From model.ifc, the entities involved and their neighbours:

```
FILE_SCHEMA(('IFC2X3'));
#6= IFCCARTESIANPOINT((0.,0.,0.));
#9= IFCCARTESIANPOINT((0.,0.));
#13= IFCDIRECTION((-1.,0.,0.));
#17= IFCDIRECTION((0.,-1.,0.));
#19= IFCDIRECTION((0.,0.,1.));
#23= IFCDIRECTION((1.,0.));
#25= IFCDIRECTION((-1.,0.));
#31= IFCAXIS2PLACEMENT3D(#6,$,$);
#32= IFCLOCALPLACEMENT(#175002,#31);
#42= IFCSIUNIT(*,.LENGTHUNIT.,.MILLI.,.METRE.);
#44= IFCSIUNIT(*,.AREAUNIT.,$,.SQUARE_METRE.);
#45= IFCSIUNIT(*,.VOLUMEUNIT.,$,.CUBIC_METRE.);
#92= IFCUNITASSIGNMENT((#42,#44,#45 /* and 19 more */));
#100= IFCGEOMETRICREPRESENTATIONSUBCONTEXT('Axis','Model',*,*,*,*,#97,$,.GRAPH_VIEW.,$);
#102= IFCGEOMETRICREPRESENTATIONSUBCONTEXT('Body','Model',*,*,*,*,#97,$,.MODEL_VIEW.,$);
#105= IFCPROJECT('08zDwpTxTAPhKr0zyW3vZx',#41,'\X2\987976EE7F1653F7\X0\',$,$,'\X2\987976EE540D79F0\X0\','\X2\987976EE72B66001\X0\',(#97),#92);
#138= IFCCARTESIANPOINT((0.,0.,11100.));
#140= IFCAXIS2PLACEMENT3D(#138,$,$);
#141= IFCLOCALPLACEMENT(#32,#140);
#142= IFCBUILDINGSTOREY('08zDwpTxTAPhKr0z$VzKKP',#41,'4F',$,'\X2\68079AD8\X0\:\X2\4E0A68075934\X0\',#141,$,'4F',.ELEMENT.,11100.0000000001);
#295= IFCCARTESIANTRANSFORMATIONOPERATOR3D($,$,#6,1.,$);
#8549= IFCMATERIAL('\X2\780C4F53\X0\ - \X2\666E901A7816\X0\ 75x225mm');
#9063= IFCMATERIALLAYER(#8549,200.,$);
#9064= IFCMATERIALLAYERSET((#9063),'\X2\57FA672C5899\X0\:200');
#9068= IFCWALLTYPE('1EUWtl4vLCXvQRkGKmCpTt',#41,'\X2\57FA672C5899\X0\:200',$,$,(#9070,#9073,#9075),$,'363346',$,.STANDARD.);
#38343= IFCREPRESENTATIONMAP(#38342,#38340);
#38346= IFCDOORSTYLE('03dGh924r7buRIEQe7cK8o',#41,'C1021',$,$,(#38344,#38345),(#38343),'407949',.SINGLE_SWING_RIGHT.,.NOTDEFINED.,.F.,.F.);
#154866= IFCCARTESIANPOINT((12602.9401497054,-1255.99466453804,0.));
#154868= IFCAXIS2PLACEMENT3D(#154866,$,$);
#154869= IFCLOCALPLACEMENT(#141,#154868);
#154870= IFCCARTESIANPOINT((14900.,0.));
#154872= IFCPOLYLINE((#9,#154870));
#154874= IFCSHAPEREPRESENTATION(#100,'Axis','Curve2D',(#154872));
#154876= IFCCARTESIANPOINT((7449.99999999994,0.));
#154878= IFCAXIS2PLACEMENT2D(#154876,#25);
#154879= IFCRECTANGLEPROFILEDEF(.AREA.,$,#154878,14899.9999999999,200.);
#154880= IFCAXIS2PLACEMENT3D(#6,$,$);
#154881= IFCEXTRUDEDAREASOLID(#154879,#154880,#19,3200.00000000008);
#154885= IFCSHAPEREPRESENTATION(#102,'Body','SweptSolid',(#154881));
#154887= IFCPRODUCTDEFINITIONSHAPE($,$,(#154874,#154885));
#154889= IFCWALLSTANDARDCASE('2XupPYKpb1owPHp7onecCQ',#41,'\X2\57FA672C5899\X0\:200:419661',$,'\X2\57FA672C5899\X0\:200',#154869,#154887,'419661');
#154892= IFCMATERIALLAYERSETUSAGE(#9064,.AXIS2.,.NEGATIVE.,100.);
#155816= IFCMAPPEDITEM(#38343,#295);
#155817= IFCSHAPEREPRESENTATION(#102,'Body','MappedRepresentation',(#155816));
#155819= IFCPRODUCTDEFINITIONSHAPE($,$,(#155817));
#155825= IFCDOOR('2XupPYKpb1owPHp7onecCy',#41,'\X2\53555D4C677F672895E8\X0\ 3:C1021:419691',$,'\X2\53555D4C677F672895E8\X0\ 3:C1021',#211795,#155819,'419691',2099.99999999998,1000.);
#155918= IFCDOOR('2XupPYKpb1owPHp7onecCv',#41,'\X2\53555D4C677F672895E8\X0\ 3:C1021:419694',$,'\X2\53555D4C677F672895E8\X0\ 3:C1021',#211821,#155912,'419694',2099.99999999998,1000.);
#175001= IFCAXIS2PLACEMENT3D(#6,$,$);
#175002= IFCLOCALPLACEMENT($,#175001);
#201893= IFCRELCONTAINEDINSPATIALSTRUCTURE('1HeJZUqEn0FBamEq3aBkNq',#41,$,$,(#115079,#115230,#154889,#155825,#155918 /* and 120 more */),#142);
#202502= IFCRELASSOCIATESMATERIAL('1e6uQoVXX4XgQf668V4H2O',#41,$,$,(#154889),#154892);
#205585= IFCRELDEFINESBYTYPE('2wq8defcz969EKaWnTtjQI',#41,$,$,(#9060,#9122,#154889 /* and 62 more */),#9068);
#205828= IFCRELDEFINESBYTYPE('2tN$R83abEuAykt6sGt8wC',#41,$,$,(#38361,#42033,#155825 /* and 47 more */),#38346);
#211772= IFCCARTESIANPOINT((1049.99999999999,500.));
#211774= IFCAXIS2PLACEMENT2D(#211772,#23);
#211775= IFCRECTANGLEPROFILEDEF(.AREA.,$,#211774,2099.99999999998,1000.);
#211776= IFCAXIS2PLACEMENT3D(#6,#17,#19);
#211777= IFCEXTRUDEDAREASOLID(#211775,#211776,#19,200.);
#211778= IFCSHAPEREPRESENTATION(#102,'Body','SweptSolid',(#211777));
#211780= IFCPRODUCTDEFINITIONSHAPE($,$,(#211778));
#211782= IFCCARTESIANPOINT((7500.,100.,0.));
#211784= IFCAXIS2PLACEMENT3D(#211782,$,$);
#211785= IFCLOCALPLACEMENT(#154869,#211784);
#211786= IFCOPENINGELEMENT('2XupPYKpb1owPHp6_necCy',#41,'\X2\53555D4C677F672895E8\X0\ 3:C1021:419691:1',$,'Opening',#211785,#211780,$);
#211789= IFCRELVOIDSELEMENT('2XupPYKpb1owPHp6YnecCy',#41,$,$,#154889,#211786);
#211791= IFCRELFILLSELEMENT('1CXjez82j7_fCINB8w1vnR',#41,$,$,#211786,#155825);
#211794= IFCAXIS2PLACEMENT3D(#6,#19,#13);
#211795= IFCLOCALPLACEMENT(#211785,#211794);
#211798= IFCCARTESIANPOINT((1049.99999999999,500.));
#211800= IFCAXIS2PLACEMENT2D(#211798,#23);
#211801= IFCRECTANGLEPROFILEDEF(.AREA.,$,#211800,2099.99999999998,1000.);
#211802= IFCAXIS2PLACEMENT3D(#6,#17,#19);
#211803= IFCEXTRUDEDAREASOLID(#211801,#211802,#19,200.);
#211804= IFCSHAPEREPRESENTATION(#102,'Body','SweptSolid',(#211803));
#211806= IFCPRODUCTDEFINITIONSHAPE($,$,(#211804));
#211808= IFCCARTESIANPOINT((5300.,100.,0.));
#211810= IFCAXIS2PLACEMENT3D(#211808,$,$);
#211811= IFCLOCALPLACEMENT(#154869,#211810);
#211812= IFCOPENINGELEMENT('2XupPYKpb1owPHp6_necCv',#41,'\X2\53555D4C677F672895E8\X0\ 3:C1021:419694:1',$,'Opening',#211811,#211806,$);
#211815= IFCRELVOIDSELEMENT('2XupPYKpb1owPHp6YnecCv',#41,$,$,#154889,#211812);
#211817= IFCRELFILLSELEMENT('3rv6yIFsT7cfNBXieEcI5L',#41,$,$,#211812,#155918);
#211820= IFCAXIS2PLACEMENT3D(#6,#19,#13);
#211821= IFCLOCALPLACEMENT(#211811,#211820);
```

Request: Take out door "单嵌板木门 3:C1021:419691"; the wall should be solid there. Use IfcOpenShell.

```python
import ifcopenshell
import ifcopenshell.api.feature
import ifcopenshell.api.root
import ifcopenshell.geom
import ifcopenshell.util.shape

model = ifcopenshell.open("model.ifc")
settings = ifcopenshell.geom.settings()


def volume(element):
    """Net volume in cubic metres, openings subtracted."""
    shape = ifcopenshell.geom.create_shape(settings, element)
    return ifcopenshell.util.shape.get_volume(shape.geometry)


door = model.by_guid("2XupPYKpb1owPHp7onecCy")
opening = door.FillsVoids[0].RelatingOpeningElement
wall = opening.VoidsElements[0].RelatingBuildingElement
before = volume(wall)

ifcopenshell.api.root.remove_product(model, product=door)
ifcopenshell.api.feature.remove_feature(model, feature=opening)

after = volume(wall)

print(f"wall volume {before:.3f} -> {after:.3f} m3")

model.write("model_updated.ifc")
```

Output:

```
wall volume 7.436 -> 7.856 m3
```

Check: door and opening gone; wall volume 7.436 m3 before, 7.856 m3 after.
